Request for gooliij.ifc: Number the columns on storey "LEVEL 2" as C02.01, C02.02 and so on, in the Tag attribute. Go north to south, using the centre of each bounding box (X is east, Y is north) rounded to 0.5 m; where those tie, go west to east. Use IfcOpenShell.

First a look at what the model holds.

```python
import ifcopenshell
import ifcopenshell.util.element
import ifcopenshell.util.placement

model = ifcopenshell.open("gooliij.ifc")
print(model.schema)
storey = next(s for s in model.by_type("IfcBuildingStorey") if s.Name == "LEVEL 2")
columns = [e for e in ifcopenshell.util.element.get_decomposition(storey) if e.is_a("IfcColumn")]
for e in sorted(columns, key=lambda e: e.id()):
    origin = ifcopenshell.util.placement.get_local_placement(e.ObjectPlacement)[:3, 3]
    print(e.id(), e.Tag, e.Name, origin.round(2) + 0.0, sep=" | ")
```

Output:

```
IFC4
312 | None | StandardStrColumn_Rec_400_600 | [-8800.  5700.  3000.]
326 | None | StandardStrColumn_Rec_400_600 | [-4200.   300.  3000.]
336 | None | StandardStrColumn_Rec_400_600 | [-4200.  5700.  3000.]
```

```python
import ifcopenshell
import ifcopenshell.geom
import ifcopenshell.util.element
import ifcopenshell.util.shape

model = ifcopenshell.open("gooliij.ifc")
settings = ifcopenshell.geom.settings()
settings.set("use-world-coords", True)


def centre(element):
    shape = ifcopenshell.geom.create_shape(settings, element)
    return ifcopenshell.util.shape.get_bbox_centroid(shape.geometry)


storey = next(s for s in model.by_type("IfcBuildingStorey") if s.Name == "LEVEL 2")
columns = [e for e in ifcopenshell.util.element.get_decomposition(storey) if e.is_a("IfcColumn")]

# Insertion points can sit at a corner or the storey origin, so sort by the geometry (in metres).
centres = {e: centre(e) for e in columns}
columns.sort(key=lambda e: (-round(centres[e][1] / 0.5), centres[e][0]))

for i, e in enumerate(columns, start=1):
    number = f"C02.{i:02d}"
    e.Tag = number
    print(e.id(), number)

model.write("gooliij_edited.ifc")
```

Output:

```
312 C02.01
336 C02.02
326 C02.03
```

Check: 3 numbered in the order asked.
